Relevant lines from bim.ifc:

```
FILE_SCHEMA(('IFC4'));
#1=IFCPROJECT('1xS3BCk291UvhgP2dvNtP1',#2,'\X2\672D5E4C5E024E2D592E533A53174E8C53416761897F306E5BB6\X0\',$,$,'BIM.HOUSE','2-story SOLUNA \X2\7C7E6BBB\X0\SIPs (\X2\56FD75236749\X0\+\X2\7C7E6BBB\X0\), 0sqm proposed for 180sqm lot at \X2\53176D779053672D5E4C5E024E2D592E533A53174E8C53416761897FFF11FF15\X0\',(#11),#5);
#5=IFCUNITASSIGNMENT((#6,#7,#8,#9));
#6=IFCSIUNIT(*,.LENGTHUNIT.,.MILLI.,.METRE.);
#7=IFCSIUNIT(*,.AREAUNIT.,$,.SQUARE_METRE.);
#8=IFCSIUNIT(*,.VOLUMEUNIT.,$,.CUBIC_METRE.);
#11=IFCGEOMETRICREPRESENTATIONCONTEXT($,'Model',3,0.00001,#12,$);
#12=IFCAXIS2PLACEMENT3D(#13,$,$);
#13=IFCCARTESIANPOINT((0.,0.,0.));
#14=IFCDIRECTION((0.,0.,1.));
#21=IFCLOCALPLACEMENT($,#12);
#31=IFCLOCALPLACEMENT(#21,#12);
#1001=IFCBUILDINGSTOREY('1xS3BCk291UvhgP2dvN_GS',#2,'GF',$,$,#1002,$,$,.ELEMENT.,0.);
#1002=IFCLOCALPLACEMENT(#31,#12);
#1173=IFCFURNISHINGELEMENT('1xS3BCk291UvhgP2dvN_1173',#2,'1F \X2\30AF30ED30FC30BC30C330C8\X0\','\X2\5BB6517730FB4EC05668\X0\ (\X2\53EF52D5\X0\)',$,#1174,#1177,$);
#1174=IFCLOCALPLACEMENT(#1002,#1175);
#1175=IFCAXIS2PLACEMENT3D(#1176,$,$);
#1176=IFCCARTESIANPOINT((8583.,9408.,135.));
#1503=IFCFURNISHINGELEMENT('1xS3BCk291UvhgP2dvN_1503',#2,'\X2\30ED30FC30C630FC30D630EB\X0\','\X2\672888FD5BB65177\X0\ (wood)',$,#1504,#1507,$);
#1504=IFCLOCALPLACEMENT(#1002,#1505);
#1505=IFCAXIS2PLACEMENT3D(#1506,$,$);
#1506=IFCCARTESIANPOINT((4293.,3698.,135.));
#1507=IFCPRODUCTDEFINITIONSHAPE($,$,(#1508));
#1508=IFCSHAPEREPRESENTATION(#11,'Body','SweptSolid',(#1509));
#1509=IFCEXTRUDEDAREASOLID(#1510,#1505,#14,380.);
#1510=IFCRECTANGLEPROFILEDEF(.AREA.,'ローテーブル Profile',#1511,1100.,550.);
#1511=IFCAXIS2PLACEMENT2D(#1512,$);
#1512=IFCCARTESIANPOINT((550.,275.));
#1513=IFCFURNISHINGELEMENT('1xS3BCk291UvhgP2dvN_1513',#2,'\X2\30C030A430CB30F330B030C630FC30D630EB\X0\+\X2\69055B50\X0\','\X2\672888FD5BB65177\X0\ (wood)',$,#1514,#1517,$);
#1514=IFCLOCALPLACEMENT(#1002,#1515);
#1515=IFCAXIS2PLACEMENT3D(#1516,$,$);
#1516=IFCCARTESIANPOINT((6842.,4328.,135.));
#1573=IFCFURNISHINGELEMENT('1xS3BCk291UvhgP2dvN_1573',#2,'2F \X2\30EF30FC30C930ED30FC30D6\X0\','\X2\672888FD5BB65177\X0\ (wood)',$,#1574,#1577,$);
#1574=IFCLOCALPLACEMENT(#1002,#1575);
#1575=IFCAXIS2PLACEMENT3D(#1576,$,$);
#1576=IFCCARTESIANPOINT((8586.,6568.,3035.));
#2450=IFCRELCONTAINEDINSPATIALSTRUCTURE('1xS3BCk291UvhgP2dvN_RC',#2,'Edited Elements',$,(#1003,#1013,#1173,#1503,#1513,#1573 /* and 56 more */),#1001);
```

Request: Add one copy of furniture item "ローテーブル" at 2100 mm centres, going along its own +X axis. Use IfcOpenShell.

```python
import ifcopenshell
import ifcopenshell.api.geometry
import ifcopenshell.api.root
import ifcopenshell.util.element
import ifcopenshell.util.placement

model = ifcopenshell.open("bim.ifc")


def reuse_history(source, copy):
    """copy_class also copies each property set's owner history, people and application; keep the originals."""
    for rel in copy.IsDefinedBy:
        if rel.is_a("IfcRelDefinesByProperties") and (history := rel.RelatingPropertyDefinition.OwnerHistory):
            rel.RelatingPropertyDefinition.OwnerHistory = source.OwnerHistory
            ifcopenshell.util.element.remove_deep2(model, history)


source = model.by_guid("1xS3BCk291UvhgP2dvN_1503")
base = ifcopenshell.util.placement.get_local_placement(source.ObjectPlacement)
step = base[:3, 0] * 2100.0

for i in range(1, 2):
    copy = ifcopenshell.api.root.copy_class(model, product=source)
    copy.Representation = ifcopenshell.util.element.copy_deep(
        model, source.Representation, exclude=["IfcGeometricRepresentationContext", "IfcRepresentationMap"]
    )
    reuse_history(source, copy)
    matrix = base.copy()
    matrix[:3, 3] += i * step
    print("added at", matrix[:3, 3].round(3) + 0.0)
    ifcopenshell.api.geometry.edit_object_placement(model, product=copy, matrix=matrix, is_si=False)

model.write("bim_rev.ifc")
```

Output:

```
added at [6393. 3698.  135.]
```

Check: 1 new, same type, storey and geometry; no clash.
